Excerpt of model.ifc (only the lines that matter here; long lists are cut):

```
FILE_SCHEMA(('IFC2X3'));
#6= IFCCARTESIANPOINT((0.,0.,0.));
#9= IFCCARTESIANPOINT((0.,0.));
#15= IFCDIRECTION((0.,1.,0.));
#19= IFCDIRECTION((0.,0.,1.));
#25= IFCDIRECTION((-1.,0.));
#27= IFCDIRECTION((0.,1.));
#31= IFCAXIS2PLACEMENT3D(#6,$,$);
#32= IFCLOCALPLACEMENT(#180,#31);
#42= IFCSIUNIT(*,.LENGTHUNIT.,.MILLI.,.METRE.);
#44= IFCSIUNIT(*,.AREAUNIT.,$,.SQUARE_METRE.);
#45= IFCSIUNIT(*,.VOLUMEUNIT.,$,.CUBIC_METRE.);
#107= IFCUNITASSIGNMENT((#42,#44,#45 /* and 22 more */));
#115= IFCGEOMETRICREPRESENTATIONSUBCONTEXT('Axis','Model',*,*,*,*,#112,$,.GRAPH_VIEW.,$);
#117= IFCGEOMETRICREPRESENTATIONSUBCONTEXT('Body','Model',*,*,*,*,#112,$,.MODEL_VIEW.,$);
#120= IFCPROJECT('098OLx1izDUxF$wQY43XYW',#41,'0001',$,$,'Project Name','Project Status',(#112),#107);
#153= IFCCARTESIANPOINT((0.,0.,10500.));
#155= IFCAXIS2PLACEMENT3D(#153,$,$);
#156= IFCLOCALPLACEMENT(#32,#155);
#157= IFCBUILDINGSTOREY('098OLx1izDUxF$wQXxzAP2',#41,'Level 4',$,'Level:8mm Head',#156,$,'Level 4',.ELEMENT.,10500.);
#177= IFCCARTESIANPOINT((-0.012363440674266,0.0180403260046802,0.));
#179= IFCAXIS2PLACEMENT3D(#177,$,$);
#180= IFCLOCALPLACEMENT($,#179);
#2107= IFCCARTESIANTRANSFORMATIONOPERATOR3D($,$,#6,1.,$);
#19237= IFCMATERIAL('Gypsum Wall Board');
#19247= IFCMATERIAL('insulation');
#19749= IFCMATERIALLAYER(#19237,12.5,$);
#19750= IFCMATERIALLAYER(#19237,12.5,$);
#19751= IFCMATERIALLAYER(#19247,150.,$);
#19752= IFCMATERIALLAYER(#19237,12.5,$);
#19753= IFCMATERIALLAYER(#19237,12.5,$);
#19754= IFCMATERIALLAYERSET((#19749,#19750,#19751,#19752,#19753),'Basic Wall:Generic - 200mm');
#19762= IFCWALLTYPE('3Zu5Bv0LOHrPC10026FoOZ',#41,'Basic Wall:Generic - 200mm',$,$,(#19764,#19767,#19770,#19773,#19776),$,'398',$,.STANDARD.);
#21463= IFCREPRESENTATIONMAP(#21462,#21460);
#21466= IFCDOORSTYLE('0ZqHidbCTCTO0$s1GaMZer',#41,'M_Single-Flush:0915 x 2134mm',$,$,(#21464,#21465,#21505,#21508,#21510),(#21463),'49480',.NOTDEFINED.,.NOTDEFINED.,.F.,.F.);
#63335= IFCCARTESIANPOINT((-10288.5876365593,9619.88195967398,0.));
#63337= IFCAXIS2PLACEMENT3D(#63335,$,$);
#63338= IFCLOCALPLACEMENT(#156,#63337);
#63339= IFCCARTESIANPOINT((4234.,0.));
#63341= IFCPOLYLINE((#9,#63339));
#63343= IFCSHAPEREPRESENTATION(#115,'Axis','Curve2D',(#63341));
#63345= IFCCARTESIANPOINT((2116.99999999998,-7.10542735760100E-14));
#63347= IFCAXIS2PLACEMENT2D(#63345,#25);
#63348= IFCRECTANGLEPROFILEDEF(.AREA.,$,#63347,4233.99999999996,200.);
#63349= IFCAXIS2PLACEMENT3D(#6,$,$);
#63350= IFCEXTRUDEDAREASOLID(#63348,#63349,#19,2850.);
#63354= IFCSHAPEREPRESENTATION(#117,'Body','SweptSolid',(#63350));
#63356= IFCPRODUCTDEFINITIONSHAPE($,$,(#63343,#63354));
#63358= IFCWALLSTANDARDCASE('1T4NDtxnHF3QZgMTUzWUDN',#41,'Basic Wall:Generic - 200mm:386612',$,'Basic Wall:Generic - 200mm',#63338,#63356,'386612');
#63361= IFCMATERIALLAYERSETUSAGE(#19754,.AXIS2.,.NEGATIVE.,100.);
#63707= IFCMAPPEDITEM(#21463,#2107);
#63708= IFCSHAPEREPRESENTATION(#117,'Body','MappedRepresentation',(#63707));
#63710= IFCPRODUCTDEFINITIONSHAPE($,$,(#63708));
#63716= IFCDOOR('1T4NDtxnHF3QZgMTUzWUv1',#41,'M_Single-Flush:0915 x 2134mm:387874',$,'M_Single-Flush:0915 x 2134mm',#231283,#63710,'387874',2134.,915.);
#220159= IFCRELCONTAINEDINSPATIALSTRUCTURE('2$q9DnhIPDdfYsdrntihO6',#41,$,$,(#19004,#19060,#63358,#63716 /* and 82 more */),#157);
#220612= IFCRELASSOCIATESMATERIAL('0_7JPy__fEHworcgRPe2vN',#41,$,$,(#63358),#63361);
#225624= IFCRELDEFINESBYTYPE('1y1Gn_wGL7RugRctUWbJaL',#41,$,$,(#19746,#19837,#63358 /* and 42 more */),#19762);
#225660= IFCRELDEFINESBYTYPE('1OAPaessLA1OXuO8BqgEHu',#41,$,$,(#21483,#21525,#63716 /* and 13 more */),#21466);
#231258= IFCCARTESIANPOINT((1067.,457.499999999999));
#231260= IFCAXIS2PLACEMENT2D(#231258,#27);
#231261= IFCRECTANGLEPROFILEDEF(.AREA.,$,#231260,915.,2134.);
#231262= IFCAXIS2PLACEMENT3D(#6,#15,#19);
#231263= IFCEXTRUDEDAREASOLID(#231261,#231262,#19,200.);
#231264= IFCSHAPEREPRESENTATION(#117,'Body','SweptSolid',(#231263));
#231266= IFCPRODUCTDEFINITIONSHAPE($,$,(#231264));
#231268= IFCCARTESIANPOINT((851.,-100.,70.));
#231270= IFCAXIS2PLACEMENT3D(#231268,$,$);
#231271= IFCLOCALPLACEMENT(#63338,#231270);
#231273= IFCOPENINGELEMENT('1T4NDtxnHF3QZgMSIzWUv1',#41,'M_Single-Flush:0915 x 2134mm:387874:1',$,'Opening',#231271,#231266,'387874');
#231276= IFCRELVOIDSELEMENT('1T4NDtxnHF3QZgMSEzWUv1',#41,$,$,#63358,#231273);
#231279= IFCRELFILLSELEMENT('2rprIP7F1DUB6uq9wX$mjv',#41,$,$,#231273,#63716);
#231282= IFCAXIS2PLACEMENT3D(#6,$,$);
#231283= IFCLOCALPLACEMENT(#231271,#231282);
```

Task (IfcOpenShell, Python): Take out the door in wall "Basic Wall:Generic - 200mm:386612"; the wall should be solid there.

```python
import ifcopenshell
import ifcopenshell.api.feature
import ifcopenshell.api.root
import ifcopenshell.geom
import ifcopenshell.util.shape

model = ifcopenshell.open("model.ifc")
settings = ifcopenshell.geom.settings()


def volume(element):
    """Net volume in cubic metres, openings subtracted."""
    shape = ifcopenshell.geom.create_shape(settings, element)
    return ifcopenshell.util.shape.get_volume(shape.geometry)


door = model.by_id(63716)
opening = door.FillsVoids[0].RelatingOpeningElement
wall = opening.VoidsElements[0].RelatingBuildingElement
before = volume(wall)

ifcopenshell.api.root.remove_product(model, product=door)
ifcopenshell.api.feature.remove_feature(model, feature=opening)

after = volume(wall)

print(f"wall volume {before:.3f} -> {after:.3f} m3")

model.write("model_updated.ifc")
```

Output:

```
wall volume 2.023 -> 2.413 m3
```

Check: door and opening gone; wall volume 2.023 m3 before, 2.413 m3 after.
